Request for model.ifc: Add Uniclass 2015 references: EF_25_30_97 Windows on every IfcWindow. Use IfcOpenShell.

First a look at what the model holds.

```python
import ifcopenshell

model = ifcopenshell.open("model.ifc")
print(model.schema)
print("classifications:", [c.Name for c in model.by_type("IfcClassification")])
for ifc_class in ("IfcDoor", "IfcRoof", "IfcStair", "IfcWall", "IfcWindow"):
    print(ifc_class, len(model.by_type(ifc_class)))
```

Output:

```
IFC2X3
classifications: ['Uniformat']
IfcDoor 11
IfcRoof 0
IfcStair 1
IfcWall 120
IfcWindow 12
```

```python
import ifcopenshell
import ifcopenshell.api.classification

model = ifcopenshell.open("model.ifc")

# IFC2X3 requires Source and Edition and has no link from the project to the system.
system = model.create_entity("IfcClassification", Source="NBS", Edition="2015", Name="Uniclass 2015")

codes = {
    "IfcWindow": ("EF_25_30_97", "Windows"),
}
for ifc_class, (code, name) in codes.items():
    products = model.by_type(ifc_class)
    ifcopenshell.api.classification.add_reference(
        model, products=products, classification=system, identification=code, name=name
    )
    print(code, len(products))

model.write("model-out.ifc")
```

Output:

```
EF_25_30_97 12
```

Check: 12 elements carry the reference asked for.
